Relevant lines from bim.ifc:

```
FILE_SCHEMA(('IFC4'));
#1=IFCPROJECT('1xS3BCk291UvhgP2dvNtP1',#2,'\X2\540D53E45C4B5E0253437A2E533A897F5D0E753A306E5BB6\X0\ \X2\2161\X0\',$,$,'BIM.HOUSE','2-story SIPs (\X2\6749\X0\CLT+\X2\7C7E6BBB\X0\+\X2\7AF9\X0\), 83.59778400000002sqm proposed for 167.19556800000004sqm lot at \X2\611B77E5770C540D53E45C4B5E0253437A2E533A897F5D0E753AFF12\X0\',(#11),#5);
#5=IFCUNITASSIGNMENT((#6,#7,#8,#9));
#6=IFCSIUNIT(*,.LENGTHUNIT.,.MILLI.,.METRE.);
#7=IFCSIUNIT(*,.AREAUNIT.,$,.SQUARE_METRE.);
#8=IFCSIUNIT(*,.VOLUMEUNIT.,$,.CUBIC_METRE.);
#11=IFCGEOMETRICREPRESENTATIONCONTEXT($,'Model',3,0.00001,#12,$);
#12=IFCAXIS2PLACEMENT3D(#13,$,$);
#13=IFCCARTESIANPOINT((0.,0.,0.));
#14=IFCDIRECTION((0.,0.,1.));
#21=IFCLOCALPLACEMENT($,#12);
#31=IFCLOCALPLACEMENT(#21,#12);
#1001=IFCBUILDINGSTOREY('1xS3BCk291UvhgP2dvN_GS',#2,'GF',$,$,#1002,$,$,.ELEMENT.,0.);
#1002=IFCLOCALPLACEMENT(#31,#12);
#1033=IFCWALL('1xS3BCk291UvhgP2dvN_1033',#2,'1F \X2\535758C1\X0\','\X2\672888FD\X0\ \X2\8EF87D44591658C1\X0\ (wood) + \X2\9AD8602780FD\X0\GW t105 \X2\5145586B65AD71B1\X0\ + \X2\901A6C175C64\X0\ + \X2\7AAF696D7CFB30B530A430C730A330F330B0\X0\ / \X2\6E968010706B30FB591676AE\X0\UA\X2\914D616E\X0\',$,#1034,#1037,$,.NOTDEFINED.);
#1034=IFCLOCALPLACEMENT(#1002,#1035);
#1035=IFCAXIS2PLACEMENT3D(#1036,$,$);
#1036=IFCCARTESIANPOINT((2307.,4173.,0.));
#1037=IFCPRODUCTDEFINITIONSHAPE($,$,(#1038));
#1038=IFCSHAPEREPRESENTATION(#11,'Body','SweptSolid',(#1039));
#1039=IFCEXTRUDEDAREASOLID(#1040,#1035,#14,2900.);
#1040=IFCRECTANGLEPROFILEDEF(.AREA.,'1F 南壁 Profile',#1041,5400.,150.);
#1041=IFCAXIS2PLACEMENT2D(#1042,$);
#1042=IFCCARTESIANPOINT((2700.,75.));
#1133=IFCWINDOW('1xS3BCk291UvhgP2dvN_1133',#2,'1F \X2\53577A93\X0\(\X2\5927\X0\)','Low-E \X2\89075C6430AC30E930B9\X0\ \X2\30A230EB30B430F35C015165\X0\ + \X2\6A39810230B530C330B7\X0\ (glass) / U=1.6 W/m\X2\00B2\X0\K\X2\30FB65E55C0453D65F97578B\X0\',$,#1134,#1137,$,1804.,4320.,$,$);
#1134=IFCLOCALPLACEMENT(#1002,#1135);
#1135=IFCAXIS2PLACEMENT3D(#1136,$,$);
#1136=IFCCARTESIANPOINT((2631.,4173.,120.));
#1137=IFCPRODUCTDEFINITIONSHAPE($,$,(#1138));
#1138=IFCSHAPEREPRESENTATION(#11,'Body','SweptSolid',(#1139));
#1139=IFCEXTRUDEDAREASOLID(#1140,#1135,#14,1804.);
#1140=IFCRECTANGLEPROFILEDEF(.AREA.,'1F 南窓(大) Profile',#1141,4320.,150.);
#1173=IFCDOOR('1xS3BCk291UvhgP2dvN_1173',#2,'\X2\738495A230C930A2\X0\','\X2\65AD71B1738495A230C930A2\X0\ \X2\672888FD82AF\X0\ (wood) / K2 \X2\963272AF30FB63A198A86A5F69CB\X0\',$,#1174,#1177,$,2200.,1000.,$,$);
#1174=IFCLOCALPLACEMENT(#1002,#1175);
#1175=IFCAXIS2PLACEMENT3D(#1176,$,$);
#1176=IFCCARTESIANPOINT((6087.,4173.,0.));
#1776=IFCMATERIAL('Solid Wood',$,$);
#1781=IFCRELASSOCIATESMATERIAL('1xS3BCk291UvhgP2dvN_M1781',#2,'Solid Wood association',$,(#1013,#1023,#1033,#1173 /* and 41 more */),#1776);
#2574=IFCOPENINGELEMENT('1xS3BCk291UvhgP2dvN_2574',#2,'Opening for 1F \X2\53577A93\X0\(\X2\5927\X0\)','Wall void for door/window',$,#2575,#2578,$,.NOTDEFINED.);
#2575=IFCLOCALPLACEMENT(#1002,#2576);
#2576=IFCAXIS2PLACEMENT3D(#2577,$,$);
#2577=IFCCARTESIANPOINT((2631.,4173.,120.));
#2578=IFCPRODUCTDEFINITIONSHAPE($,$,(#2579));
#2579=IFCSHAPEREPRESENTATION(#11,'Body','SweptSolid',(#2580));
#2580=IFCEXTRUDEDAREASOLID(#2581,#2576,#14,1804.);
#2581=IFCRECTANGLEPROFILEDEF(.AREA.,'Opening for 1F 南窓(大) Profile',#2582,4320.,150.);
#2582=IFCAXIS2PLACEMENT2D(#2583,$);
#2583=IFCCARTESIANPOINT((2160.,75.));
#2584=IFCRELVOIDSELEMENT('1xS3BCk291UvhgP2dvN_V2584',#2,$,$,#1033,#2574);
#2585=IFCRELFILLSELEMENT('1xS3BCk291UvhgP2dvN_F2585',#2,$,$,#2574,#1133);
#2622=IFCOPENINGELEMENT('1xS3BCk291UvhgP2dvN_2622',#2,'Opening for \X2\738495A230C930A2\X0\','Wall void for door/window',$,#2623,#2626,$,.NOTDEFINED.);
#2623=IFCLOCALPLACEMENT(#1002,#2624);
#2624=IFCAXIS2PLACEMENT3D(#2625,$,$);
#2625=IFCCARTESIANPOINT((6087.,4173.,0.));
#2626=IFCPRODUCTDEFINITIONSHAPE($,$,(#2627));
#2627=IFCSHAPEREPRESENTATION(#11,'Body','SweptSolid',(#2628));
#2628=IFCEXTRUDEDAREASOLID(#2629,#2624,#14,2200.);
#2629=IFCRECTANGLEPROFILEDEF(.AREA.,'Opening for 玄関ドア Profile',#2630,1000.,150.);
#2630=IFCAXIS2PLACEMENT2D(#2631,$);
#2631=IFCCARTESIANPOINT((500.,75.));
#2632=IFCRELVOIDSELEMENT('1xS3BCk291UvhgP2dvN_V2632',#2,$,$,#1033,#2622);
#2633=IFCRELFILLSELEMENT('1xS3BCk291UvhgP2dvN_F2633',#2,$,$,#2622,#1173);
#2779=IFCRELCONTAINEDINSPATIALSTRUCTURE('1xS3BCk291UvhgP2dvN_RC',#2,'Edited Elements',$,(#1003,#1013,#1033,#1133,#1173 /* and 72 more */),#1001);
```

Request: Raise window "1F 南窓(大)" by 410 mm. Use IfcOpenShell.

```python
import numpy as np
import ifcopenshell
import ifcopenshell.api.geometry
import ifcopenshell.util.placement
import ifcopenshell.util.unit

model = ifcopenshell.open("bim.ifc")
unit_scale = ifcopenshell.util.unit.calculate_unit_scale(model)

window = model.by_guid("1xS3BCk291UvhgP2dvN_1133")
opening = window.FillsVoids[0].RelatingOpeningElement
dz = 0.41 / unit_scale

shift = np.array([0.0, 0.0, dz])
# The window is not placed relative to its opening, so move both.
for product in (opening, window):
    matrix = ifcopenshell.util.placement.get_local_placement(product.ObjectPlacement)
    matrix[:3, 3] += shift
    ifcopenshell.api.geometry.edit_object_placement(model, product=product, matrix=matrix, is_si=False)

print(f"moved by {dz * unit_scale:+.3f} m")

model.write("bim_rev.ifc")
```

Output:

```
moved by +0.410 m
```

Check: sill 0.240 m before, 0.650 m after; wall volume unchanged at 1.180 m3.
